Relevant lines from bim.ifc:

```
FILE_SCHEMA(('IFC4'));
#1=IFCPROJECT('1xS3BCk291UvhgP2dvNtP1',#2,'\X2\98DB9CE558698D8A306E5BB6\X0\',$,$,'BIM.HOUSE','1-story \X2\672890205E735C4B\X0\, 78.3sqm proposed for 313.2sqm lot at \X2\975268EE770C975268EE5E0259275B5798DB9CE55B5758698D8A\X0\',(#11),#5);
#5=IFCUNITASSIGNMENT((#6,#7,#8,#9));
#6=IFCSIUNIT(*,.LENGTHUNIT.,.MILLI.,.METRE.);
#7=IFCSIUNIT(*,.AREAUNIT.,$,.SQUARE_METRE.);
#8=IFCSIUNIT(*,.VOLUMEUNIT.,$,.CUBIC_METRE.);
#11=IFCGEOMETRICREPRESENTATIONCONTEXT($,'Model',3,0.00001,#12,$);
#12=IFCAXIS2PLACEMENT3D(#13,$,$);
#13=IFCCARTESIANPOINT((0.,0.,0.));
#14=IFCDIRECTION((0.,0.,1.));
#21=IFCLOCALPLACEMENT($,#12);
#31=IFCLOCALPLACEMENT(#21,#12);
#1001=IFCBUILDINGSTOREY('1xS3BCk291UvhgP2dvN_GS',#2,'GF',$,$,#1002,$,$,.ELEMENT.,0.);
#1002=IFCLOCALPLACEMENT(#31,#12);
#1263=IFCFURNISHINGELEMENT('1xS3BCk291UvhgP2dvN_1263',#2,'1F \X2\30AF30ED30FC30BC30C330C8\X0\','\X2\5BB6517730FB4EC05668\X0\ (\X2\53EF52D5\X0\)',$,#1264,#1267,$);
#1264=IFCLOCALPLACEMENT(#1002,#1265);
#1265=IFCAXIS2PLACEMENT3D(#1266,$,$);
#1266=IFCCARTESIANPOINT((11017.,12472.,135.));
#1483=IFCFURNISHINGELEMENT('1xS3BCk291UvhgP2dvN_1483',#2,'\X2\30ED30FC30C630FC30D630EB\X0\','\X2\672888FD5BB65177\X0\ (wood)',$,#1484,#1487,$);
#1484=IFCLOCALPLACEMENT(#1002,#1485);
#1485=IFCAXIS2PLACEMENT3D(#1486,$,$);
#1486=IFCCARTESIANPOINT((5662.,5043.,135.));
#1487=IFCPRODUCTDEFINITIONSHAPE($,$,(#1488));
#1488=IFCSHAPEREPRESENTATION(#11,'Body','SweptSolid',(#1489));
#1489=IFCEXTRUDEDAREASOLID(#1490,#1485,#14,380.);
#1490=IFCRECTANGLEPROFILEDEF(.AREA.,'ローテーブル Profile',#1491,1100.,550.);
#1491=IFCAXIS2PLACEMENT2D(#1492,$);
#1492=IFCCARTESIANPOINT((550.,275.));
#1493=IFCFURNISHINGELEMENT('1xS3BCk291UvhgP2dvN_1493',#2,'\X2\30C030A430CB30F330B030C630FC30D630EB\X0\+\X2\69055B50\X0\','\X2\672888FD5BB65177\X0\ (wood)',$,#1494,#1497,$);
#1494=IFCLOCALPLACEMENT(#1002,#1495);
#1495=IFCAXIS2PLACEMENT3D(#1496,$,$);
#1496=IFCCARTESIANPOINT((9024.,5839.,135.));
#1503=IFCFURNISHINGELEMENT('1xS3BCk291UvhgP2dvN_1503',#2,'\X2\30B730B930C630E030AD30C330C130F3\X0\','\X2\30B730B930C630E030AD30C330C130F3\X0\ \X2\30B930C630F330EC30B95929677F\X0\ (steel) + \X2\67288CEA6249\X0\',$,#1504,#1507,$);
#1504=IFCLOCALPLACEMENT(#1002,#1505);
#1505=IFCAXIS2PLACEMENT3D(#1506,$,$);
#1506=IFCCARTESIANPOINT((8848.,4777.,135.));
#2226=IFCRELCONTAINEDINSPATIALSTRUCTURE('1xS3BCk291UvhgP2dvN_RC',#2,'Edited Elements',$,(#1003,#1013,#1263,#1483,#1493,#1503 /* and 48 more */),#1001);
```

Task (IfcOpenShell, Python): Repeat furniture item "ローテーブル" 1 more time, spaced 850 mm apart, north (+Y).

```python
import numpy as np
import ifcopenshell
import ifcopenshell.api.geometry
import ifcopenshell.api.root
import ifcopenshell.util.element
import ifcopenshell.util.placement
import ifcopenshell.util.unit

model = ifcopenshell.open("bim.ifc")
unit_scale = ifcopenshell.util.unit.calculate_unit_scale(model)


def reuse_history(source, copy):
    """copy_class also copies each property set's owner history, people and application; keep the originals."""
    for rel in copy.IsDefinedBy:
        if rel.is_a("IfcRelDefinesByProperties") and (history := rel.RelatingPropertyDefinition.OwnerHistory):
            rel.RelatingPropertyDefinition.OwnerHistory = source.OwnerHistory
            ifcopenshell.util.element.remove_deep2(model, history)


source = model.by_guid("1xS3BCk291UvhgP2dvN_1483")
base = ifcopenshell.util.placement.get_local_placement(source.ObjectPlacement)
step = np.array([0.0, 1.0, 0.0]) * 0.85 / unit_scale

for i in range(1, 2):
    copy = ifcopenshell.api.root.copy_class(model, product=source)
    copy.Representation = ifcopenshell.util.element.copy_deep(
        model, source.Representation, exclude=["IfcGeometricRepresentationContext", "IfcRepresentationMap"]
    )
    reuse_history(source, copy)
    matrix = base.copy()
    matrix[:3, 3] += i * step
    print("added at", matrix[:3, 3].round(3) + 0.0)
    ifcopenshell.api.geometry.edit_object_placement(model, product=copy, matrix=matrix, is_si=False)

model.write("bim_edited.ifc")
```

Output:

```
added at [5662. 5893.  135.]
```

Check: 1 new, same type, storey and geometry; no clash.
